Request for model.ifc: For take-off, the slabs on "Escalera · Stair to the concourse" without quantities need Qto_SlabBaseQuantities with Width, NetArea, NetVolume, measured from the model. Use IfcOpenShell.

First a look at what the model holds.

```python
import ifcopenshell
import ifcopenshell.util.element
import ifcopenshell.util.unit

model = ifcopenshell.open("model.ifc")
print(model.schema)
for unit_type in ("LENGTHUNIT", "AREAUNIT", "VOLUMEUNIT"):
    print(unit_type, ifcopenshell.util.unit.calculate_unit_scale(model, unit_type))
storey = next(s for s in model.by_type("IfcBuildingStorey") if s.Name == "Escalera · Stair to the concourse")
slabs = [e for e in ifcopenshell.util.element.get_decomposition(storey) if e.is_a("IfcSlab")]
for e in sorted(slabs, key=lambda e: e.id()):
    print(e.id(), e.is_a(), e.Name, list(ifcopenshell.util.element.get_psets(e, qtos_only=True)), sep=" | ")
```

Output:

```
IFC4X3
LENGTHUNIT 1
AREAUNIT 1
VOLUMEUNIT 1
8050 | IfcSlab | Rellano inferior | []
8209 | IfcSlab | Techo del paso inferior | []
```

```python
import ifcopenshell
import ifcopenshell.api.pset
import ifcopenshell.geom
import ifcopenshell.util.element
import ifcopenshell.util.shape
import ifcopenshell.util.unit

model = ifcopenshell.open("model.ifc")
unit_scale = ifcopenshell.util.unit.calculate_unit_scale(model)
area_scale = ifcopenshell.util.unit.calculate_unit_scale(model, "AREAUNIT")
volume_scale = ifcopenshell.util.unit.calculate_unit_scale(model, "VOLUMEUNIT")
settings = ifcopenshell.geom.settings()

storey = next(s for s in model.by_type("IfcBuildingStorey") if s.Name == "Escalera · Stair to the concourse")
slabs = [e for e in ifcopenshell.util.element.get_decomposition(storey) if e.is_a("IfcSlab")]

for e in sorted(slabs, key=lambda e: e.id()):
    if ifcopenshell.util.element.get_psets(e, qtos_only=True, should_inherit=False):
        continue
    # Geometry comes back in metres, in the element's own axes.
    shape = ifcopenshell.geom.create_shape(settings, e)
    values = {
        "Width": ifcopenshell.util.shape.get_z(shape.geometry) / unit_scale,
        "NetArea": ifcopenshell.util.shape.get_footprint_area(shape.geometry) / area_scale,
        "NetVolume": ifcopenshell.util.shape.get_volume(shape.geometry) / volume_scale,
    }
    qto = ifcopenshell.api.pset.add_qto(model, product=e, name="Qto_SlabBaseQuantities")
    ifcopenshell.api.pset.edit_qto(model, qto=qto, properties=values)
    print(e.id(), {k: round(v, 3) for k, v in values.items()})

model.write("model_edited.ifc")
```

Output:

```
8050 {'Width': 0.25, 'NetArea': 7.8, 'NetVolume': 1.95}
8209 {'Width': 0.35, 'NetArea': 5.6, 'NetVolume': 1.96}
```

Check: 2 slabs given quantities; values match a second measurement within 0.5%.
